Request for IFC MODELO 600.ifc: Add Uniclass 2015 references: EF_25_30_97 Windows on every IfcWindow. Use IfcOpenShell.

First a look at what the model holds.

```python
import ifcopenshell

model = ifcopenshell.open("IFC MODELO 600.ifc")
print(model.schema)
print("classifications:", [c.Name for c in model.by_type("IfcClassification")])
for ifc_class in ("IfcDoor", "IfcRoof", "IfcStair", "IfcWall", "IfcWindow"):
    print(ifc_class, len(model.by_type(ifc_class)))
```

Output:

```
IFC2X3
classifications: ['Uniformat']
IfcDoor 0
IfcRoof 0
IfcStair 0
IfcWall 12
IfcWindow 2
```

```python
import ifcopenshell
import ifcopenshell.api.classification

model = ifcopenshell.open("IFC MODELO 600.ifc")

# IFC2X3 requires Source and Edition and has no link from the project to the system.
system = model.create_entity("IfcClassification", Source="NBS", Edition="2015", Name="Uniclass 2015")

codes = {
    "IfcWindow": ("EF_25_30_97", "Windows"),
}
for ifc_class, (code, name) in codes.items():
    products = model.by_type(ifc_class)
    ifcopenshell.api.classification.add_reference(
        model, products=products, classification=system, identification=code, name=name
    )
    print(code, len(products))

model.write("IFC MODELO 600_rev.ifc")
```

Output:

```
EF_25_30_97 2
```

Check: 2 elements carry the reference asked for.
